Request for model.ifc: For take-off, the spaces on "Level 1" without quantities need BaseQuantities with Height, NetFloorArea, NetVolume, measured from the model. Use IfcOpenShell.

First a look at what the model holds.

```python
import ifcopenshell
import ifcopenshell.util.element
import ifcopenshell.util.unit

model = ifcopenshell.open("model.ifc")
print(model.schema)
for unit_type in ("LENGTHUNIT", "AREAUNIT", "VOLUMEUNIT"):
    print(unit_type, ifcopenshell.util.unit.calculate_unit_scale(model, unit_type))
storey = next(s for s in model.by_type("IfcBuildingStorey") if s.Name == "Level 1")
spaces = [e for e in ifcopenshell.util.element.get_decomposition(storey) if e.is_a("IfcSpace")]
for e in sorted(spaces, key=lambda e: e.id()):
    print(e.id(), e.is_a(), e.Name, list(ifcopenshell.util.element.get_psets(e, qtos_only=True)), sep=" | ")
```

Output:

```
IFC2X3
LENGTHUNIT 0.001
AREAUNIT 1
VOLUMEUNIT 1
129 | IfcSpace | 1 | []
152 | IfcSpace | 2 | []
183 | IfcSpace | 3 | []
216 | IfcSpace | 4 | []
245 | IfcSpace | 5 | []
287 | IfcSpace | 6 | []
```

```python
import ifcopenshell
import ifcopenshell.api.pset
import ifcopenshell.geom
import ifcopenshell.util.element
import ifcopenshell.util.shape
import ifcopenshell.util.unit

model = ifcopenshell.open("model.ifc")
unit_scale = ifcopenshell.util.unit.calculate_unit_scale(model)
area_scale = ifcopenshell.util.unit.calculate_unit_scale(model, "AREAUNIT")
volume_scale = ifcopenshell.util.unit.calculate_unit_scale(model, "VOLUMEUNIT")
settings = ifcopenshell.geom.settings()

storey = next(s for s in model.by_type("IfcBuildingStorey") if s.Name == "Level 1")
spaces = [e for e in ifcopenshell.util.element.get_decomposition(storey) if e.is_a("IfcSpace")]

for e in sorted(spaces, key=lambda e: e.id()):
    if ifcopenshell.util.element.get_psets(e, qtos_only=True, should_inherit=False):
        continue
    # Geometry comes back in metres, in the element's own axes.
    shape = ifcopenshell.geom.create_shape(settings, e)
    values = {
        "Height": ifcopenshell.util.shape.get_z(shape.geometry) / unit_scale,
        "NetFloorArea": ifcopenshell.util.shape.get_footprint_area(shape.geometry) / area_scale,
        "NetVolume": ifcopenshell.util.shape.get_volume(shape.geometry) / volume_scale,
    }
    qto = ifcopenshell.api.pset.add_qto(model, product=e, name="BaseQuantities")
    ifcopenshell.api.pset.edit_qto(model, qto=qto, properties=values)
    print(e.id(), {k: round(v, 3) for k, v in values.items()})

model.write("model-out.ifc")
```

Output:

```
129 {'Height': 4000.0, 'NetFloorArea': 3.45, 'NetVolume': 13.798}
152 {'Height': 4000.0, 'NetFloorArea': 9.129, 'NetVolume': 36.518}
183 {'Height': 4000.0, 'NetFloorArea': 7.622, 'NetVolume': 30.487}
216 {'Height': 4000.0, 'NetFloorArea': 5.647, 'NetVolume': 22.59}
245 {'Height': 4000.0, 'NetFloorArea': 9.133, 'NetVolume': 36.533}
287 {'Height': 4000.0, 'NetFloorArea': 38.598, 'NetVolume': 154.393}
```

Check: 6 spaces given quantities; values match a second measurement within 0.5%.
